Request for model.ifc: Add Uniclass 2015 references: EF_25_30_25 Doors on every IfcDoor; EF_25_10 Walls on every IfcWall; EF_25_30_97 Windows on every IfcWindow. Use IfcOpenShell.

First a look at what the model holds.

```python
import ifcopenshell

model = ifcopenshell.open("model.ifc")
print(model.schema)
print("classifications:", [c.Name for c in model.by_type("IfcClassification")])
for ifc_class in ("IfcDoor", "IfcRoof", "IfcStair", "IfcWall", "IfcWindow"):
    print(ifc_class, len(model.by_type(ifc_class)))
```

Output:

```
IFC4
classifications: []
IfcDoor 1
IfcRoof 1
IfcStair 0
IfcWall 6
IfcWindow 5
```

```python
import ifcopenshell
import ifcopenshell.api.classification

model = ifcopenshell.open("model.ifc")

system = ifcopenshell.api.classification.add_classification(model, classification="Uniclass 2015")

codes = {
    "IfcDoor": ("EF_25_30_25", "Doors"),
    "IfcWall": ("EF_25_10", "Walls"),
    "IfcWindow": ("EF_25_30_97", "Windows"),
}
for ifc_class, (code, name) in codes.items():
    products = model.by_type(ifc_class)
    ifcopenshell.api.classification.add_reference(
        model, products=products, classification=system, identification=code, name=name
    )
    print(code, len(products))

model.write("model_edited.ifc")
```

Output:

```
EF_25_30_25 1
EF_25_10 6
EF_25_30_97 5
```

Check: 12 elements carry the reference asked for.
